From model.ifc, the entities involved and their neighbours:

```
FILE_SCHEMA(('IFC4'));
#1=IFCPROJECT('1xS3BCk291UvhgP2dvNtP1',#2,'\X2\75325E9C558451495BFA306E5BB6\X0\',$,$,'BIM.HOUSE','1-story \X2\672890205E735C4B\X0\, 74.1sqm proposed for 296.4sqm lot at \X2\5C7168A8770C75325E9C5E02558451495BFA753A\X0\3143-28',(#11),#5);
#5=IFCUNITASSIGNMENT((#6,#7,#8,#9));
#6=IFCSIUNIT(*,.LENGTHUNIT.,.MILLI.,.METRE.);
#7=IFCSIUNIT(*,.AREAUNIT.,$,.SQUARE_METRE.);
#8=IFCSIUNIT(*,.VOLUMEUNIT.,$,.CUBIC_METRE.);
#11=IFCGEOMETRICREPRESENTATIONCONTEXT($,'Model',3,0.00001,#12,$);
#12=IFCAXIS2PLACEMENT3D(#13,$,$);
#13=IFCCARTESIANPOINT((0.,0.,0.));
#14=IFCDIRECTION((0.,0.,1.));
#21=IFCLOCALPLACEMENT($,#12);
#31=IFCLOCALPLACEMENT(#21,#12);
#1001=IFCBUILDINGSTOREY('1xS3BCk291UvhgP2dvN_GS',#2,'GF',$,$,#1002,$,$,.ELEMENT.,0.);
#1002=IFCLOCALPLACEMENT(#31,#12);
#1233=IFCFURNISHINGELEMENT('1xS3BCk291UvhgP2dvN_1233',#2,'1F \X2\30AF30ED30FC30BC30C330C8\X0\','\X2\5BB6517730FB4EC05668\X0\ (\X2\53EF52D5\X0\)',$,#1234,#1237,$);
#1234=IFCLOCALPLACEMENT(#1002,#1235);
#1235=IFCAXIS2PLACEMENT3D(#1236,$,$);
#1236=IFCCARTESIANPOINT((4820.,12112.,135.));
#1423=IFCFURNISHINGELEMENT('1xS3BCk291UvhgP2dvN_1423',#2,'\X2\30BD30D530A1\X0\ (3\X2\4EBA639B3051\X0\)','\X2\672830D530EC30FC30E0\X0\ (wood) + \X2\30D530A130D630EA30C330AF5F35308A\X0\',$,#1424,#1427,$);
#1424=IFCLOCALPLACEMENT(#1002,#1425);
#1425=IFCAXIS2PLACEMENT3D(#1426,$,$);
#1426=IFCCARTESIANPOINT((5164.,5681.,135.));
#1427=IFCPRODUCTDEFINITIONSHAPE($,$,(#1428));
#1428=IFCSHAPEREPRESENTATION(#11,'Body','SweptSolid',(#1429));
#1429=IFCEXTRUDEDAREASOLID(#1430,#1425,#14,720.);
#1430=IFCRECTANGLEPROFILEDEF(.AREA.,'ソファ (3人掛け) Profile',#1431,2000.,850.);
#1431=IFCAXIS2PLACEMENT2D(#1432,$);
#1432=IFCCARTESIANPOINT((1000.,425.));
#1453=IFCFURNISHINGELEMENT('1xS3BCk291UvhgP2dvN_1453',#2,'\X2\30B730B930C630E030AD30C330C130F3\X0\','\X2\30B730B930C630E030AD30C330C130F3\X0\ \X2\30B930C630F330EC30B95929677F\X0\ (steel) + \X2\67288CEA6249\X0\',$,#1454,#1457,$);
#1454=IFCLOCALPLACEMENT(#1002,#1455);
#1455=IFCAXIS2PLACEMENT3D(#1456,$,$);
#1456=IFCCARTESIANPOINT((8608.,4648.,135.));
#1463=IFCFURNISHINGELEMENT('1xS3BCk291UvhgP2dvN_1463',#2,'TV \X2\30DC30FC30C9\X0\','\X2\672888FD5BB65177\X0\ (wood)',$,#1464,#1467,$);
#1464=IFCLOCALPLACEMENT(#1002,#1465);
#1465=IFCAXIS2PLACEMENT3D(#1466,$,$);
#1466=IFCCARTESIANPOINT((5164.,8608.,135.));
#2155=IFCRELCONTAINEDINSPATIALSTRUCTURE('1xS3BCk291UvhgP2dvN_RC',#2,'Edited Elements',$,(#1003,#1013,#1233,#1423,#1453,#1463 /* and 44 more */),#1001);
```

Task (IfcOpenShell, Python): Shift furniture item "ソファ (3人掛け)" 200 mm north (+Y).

```python
import ifcopenshell
import ifcopenshell.api.geometry
import ifcopenshell.util.placement
import ifcopenshell.util.unit

model = ifcopenshell.open("model.ifc")
unit_scale = ifcopenshell.util.unit.calculate_unit_scale(model)

item = model.by_id(1423)
matrix = ifcopenshell.util.placement.get_local_placement(item.ObjectPlacement)
matrix[1, 3] += 0.2 / unit_scale
ifcopenshell.api.geometry.edit_object_placement(model, product=item, matrix=matrix, is_si=False)

print(ifcopenshell.util.placement.get_local_placement(item.ObjectPlacement).round(3) + 0.0)

model.write("model_edited.ifc")
```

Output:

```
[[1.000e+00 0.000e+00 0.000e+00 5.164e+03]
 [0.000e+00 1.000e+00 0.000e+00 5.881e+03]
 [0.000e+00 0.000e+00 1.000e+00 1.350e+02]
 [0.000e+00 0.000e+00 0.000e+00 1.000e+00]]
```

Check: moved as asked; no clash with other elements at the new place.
